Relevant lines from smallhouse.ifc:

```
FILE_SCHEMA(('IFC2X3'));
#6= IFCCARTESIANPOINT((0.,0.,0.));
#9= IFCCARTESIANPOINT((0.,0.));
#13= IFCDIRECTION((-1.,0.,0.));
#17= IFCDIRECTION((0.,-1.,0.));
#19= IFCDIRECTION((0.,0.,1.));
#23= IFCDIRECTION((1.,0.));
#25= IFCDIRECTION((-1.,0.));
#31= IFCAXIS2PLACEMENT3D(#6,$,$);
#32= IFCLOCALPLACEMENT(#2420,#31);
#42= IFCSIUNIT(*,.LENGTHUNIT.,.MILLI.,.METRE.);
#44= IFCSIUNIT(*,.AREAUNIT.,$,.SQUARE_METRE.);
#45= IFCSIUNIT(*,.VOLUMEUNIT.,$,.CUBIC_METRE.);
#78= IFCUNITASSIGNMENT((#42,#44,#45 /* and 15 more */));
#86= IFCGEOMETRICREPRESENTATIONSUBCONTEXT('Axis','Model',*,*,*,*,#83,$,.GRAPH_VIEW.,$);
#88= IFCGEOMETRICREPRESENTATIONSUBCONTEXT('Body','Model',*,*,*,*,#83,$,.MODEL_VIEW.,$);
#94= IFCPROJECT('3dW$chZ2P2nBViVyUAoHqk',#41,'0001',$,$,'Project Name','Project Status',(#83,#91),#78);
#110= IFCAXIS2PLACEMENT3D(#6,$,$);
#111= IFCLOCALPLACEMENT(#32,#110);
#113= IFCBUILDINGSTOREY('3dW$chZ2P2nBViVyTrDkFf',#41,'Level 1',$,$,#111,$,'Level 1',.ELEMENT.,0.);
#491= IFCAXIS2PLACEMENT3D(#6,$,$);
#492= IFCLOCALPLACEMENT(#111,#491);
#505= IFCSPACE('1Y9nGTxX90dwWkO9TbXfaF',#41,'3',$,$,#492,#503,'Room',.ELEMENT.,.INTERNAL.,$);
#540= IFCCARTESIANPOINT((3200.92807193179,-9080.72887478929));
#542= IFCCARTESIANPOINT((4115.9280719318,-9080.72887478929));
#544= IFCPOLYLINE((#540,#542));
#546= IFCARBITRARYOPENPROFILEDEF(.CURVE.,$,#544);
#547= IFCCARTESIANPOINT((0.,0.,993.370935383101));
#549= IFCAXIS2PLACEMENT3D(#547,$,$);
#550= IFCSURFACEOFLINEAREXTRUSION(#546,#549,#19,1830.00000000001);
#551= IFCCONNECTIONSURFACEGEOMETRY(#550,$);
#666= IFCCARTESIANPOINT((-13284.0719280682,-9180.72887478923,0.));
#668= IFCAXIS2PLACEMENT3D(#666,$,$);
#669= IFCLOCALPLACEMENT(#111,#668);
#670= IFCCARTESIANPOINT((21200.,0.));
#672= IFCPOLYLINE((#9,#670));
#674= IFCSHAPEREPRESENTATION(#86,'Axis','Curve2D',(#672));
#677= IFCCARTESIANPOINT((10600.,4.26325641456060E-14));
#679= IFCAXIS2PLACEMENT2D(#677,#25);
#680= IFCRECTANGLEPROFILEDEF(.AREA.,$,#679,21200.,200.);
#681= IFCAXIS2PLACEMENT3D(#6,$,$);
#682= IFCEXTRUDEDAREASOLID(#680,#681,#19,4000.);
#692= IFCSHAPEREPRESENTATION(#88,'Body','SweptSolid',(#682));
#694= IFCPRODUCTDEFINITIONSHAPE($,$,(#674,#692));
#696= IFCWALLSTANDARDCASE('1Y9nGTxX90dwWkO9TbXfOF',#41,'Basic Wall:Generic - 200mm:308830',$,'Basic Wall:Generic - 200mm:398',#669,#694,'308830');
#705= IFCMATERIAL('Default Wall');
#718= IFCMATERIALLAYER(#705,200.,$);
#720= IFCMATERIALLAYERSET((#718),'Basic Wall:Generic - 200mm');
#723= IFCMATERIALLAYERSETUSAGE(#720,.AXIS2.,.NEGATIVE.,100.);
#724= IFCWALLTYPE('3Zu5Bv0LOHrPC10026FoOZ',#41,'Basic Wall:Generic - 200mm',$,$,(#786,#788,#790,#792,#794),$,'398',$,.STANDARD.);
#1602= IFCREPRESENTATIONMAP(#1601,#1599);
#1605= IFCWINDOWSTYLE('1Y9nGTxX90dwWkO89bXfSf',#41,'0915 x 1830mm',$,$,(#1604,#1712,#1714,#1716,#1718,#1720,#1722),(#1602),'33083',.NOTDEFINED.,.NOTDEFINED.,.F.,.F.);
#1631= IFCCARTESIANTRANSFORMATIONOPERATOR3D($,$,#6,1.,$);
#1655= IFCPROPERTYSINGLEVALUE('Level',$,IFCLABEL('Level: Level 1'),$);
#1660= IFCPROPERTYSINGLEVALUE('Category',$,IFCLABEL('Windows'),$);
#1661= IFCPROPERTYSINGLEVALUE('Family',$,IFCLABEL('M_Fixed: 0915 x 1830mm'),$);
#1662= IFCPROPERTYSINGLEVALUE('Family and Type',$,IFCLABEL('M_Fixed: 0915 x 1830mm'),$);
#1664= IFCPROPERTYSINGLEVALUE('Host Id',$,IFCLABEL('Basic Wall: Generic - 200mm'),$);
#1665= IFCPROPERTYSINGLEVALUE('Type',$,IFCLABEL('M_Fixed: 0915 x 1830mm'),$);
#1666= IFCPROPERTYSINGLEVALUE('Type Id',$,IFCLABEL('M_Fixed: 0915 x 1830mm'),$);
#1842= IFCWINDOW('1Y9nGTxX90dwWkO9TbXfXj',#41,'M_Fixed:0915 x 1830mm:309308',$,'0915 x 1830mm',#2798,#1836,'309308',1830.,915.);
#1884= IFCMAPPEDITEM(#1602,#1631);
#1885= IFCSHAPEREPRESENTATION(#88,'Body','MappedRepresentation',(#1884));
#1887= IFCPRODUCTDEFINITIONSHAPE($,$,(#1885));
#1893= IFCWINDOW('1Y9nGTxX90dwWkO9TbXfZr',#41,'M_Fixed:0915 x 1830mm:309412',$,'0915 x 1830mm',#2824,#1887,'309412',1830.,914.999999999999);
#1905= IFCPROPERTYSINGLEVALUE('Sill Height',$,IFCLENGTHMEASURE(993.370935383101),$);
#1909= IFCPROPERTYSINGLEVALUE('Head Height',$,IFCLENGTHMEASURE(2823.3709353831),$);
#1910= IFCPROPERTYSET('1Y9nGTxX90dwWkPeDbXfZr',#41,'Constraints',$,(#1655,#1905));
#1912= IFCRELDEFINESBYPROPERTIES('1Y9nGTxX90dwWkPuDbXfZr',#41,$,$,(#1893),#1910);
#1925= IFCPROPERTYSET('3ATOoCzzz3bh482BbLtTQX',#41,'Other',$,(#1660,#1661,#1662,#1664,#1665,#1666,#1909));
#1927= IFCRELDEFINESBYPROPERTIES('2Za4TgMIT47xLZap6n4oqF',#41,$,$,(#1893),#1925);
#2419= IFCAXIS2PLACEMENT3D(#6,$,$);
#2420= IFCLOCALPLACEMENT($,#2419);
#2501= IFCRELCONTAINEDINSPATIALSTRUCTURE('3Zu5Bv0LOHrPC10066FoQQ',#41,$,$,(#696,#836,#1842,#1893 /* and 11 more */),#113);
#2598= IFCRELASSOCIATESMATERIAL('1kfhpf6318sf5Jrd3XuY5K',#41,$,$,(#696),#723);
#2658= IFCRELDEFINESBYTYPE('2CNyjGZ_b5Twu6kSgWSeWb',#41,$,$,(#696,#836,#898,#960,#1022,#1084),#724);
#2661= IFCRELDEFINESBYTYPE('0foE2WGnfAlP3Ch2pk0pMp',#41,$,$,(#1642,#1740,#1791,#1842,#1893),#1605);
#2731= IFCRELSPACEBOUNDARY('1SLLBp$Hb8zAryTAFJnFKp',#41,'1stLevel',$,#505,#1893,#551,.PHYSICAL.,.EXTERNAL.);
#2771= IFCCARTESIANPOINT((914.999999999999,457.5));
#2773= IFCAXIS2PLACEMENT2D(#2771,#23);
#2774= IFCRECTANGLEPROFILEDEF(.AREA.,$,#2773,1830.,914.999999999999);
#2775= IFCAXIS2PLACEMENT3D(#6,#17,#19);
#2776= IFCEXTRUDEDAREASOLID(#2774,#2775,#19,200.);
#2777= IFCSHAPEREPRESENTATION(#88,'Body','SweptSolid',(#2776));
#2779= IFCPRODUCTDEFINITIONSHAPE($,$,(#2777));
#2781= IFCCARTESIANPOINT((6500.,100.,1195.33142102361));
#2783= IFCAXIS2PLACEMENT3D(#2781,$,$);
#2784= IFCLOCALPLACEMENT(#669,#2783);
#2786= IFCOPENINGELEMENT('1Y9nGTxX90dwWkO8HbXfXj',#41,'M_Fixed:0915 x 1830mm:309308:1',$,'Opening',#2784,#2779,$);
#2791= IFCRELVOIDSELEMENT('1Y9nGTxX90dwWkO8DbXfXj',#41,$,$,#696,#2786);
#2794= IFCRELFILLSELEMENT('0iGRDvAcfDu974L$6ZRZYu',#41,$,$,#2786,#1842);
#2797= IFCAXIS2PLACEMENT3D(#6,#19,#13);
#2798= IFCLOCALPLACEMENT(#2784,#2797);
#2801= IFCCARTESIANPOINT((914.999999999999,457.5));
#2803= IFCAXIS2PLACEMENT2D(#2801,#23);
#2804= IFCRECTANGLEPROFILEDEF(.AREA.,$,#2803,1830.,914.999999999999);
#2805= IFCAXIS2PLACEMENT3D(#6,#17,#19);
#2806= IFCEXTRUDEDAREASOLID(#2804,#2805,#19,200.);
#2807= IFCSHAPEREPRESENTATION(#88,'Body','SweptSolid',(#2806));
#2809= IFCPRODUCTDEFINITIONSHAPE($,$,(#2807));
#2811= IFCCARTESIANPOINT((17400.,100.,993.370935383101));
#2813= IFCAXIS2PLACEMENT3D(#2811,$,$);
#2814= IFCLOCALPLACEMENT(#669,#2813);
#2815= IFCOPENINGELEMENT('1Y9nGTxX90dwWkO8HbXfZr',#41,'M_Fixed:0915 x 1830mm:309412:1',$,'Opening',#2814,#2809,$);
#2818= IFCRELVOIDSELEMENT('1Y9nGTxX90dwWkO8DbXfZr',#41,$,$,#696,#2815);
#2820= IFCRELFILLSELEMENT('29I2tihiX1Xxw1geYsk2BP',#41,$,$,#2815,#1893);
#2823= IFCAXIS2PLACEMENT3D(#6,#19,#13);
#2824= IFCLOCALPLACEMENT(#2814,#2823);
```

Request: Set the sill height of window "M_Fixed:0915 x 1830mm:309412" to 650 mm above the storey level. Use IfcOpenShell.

```python
import numpy as np
import ifcopenshell
import ifcopenshell.api.geometry
import ifcopenshell.api.pset
import ifcopenshell.geom
import ifcopenshell.util.element
import ifcopenshell.util.placement
import ifcopenshell.util.shape
import ifcopenshell.util.unit

model = ifcopenshell.open("smallhouse.ifc")
unit_scale = ifcopenshell.util.unit.calculate_unit_scale(model)

window = model.by_guid("1Y9nGTxX90dwWkO9TbXfZr")
opening = window.FillsVoids[0].RelatingOpeningElement
storey = ifcopenshell.util.element.get_container(window, ifc_class="IfcBuildingStorey")
level = ifcopenshell.util.placement.get_local_placement(storey.ObjectPlacement)[2, 3]

# The opening's origin need not be at the sill, so measure its lowest point.
shape = ifcopenshell.geom.create_shape(ifcopenshell.geom.settings(), opening)
bottom = ifcopenshell.util.shape.get_shape_bottom_elevation(shape, shape.geometry) / unit_scale
dz = level + 650.0 - bottom

shift = np.array([0.0, 0.0, dz])
# The window is placed relative to its opening, so it follows when the opening moves.
matrix = ifcopenshell.util.placement.get_local_placement(opening.ObjectPlacement)
matrix[:3, 3] += shift
ifcopenshell.api.geometry.edit_object_placement(
    model, product=opening, matrix=matrix, is_si=False, should_transform_children=True
)

# Space boundary surfaces are stored in each space's coordinates; move them too.
for rel in window.ProvidesBoundaries:
    if not rel.ConnectionGeometry:
        continue
    surface = rel.ConnectionGeometry.SurfaceOnRelatingElement
    space_matrix = ifcopenshell.util.placement.get_local_placement(rel.RelatingSpace.ObjectPlacement)
    point = np.array(surface.Position.Location.Coordinates) + space_matrix[:3, :3].T @ shift
    surface.Position = model.createIfcAxis2Placement3D(
        model.createIfcCartesianPoint(point.tolist()), surface.Position.Axis, surface.Position.RefDirection
    )

# Keep the stored heights in step.
pset = model.by_id(ifcopenshell.util.element.get_pset(window, "Constraints", should_inherit=False)["id"])
ifcopenshell.api.pset.edit_pset(model, pset=pset, properties={
    "Sill Height": model.create_entity("IfcLengthMeasure", ifcopenshell.util.element.get_pset(window, "Constraints", "Sill Height") + dz),
})
pset = model.by_id(ifcopenshell.util.element.get_pset(window, "Other", should_inherit=False)["id"])
ifcopenshell.api.pset.edit_pset(model, pset=pset, properties={
    "Head Height": model.create_entity("IfcLengthMeasure", ifcopenshell.util.element.get_pset(window, "Other", "Head Height") + dz),
})

print(f"moved by {dz * unit_scale:+.3f} m")

model.write("smallhouse_updated.ifc")
```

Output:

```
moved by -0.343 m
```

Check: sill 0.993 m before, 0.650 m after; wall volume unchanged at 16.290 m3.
